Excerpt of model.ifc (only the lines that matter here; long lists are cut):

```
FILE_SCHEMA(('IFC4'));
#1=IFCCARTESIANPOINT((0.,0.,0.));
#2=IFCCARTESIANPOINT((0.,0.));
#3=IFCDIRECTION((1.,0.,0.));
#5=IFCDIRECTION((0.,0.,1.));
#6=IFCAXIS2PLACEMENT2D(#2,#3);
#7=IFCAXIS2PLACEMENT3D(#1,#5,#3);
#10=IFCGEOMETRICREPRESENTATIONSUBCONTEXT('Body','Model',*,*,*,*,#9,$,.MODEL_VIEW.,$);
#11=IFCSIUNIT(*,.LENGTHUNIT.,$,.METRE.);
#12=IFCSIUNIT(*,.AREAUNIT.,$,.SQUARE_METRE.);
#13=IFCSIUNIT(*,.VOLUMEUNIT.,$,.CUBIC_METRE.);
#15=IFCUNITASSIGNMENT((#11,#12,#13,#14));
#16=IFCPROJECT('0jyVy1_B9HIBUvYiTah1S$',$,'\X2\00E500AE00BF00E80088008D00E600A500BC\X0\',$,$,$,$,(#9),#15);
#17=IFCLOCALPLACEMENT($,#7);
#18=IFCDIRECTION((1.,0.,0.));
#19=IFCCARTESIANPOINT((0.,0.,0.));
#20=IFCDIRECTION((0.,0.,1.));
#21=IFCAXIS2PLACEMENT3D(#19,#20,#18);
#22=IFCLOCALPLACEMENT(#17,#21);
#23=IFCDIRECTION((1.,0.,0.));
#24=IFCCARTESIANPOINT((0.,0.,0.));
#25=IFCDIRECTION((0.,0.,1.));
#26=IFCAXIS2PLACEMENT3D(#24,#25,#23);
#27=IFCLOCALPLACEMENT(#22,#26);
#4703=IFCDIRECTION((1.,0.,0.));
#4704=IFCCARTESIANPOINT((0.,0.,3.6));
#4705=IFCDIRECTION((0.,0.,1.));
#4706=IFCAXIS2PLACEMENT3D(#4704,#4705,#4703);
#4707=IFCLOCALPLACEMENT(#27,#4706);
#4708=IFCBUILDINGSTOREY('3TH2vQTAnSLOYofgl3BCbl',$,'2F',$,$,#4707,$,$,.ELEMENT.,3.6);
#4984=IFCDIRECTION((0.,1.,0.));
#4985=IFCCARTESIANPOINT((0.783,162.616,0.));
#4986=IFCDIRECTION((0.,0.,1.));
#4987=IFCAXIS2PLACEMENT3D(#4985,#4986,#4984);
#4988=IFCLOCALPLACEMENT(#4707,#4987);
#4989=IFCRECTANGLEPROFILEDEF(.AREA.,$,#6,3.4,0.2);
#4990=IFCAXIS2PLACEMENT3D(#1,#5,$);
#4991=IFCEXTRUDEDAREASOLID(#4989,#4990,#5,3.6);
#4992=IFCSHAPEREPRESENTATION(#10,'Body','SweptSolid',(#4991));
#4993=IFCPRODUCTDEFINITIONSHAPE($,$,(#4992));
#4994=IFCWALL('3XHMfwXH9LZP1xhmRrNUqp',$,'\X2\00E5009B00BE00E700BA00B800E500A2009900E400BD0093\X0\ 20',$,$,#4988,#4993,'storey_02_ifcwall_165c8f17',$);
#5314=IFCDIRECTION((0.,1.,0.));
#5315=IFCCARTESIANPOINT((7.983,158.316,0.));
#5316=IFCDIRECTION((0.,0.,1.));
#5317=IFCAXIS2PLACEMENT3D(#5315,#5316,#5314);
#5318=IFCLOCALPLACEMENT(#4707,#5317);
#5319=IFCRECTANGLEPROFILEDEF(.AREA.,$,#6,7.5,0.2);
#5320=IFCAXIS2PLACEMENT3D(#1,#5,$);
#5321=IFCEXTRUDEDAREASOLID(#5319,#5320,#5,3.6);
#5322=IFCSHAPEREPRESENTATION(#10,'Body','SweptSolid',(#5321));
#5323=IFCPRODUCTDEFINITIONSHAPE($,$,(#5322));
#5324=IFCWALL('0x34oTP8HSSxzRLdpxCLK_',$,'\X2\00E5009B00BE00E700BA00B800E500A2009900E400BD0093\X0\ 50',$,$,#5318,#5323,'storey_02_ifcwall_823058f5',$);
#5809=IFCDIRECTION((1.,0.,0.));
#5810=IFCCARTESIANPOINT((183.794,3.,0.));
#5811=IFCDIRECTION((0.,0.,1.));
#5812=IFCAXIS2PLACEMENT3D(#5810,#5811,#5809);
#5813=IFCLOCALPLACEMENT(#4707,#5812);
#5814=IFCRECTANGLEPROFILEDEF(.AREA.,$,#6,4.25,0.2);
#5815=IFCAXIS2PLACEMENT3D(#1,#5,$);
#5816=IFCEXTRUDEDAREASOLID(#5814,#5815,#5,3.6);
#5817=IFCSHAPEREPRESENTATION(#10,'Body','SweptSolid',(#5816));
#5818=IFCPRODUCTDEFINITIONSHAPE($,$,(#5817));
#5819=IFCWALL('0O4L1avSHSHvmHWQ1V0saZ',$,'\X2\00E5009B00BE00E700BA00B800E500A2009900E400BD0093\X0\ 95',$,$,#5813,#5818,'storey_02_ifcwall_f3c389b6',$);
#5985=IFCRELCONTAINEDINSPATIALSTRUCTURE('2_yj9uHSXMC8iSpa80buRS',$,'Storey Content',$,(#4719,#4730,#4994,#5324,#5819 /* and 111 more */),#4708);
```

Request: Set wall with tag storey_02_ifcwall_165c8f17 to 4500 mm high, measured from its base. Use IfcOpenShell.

```python
import ifcopenshell
import ifcopenshell.geom
import ifcopenshell.util.representation
import ifcopenshell.util.shape
import ifcopenshell.util.unit

model = ifcopenshell.open("model.ifc")
unit_scale = ifcopenshell.util.unit.calculate_unit_scale(model)
settings = ifcopenshell.geom.settings()


def volume(element):
    """Net volume in cubic metres, openings subtracted."""
    shape = ifcopenshell.geom.create_shape(settings, element)
    return ifcopenshell.util.shape.get_volume(shape.geometry)


wall = model.by_id(4994)
before = volume(wall)

body = ifcopenshell.util.representation.get_representation(wall, "Model", "Body")
solid = body.Items[0]
old_height = solid.Depth
solid.Depth = 4.5 / unit_scale
after = volume(wall)

print(f"height {old_height:g} -> {solid.Depth:g}, volume {before:.3f} -> {after:.3f} m3")

model.write("model_rev.ifc")
```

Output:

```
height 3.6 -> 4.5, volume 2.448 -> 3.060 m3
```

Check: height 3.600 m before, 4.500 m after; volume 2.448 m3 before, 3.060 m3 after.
